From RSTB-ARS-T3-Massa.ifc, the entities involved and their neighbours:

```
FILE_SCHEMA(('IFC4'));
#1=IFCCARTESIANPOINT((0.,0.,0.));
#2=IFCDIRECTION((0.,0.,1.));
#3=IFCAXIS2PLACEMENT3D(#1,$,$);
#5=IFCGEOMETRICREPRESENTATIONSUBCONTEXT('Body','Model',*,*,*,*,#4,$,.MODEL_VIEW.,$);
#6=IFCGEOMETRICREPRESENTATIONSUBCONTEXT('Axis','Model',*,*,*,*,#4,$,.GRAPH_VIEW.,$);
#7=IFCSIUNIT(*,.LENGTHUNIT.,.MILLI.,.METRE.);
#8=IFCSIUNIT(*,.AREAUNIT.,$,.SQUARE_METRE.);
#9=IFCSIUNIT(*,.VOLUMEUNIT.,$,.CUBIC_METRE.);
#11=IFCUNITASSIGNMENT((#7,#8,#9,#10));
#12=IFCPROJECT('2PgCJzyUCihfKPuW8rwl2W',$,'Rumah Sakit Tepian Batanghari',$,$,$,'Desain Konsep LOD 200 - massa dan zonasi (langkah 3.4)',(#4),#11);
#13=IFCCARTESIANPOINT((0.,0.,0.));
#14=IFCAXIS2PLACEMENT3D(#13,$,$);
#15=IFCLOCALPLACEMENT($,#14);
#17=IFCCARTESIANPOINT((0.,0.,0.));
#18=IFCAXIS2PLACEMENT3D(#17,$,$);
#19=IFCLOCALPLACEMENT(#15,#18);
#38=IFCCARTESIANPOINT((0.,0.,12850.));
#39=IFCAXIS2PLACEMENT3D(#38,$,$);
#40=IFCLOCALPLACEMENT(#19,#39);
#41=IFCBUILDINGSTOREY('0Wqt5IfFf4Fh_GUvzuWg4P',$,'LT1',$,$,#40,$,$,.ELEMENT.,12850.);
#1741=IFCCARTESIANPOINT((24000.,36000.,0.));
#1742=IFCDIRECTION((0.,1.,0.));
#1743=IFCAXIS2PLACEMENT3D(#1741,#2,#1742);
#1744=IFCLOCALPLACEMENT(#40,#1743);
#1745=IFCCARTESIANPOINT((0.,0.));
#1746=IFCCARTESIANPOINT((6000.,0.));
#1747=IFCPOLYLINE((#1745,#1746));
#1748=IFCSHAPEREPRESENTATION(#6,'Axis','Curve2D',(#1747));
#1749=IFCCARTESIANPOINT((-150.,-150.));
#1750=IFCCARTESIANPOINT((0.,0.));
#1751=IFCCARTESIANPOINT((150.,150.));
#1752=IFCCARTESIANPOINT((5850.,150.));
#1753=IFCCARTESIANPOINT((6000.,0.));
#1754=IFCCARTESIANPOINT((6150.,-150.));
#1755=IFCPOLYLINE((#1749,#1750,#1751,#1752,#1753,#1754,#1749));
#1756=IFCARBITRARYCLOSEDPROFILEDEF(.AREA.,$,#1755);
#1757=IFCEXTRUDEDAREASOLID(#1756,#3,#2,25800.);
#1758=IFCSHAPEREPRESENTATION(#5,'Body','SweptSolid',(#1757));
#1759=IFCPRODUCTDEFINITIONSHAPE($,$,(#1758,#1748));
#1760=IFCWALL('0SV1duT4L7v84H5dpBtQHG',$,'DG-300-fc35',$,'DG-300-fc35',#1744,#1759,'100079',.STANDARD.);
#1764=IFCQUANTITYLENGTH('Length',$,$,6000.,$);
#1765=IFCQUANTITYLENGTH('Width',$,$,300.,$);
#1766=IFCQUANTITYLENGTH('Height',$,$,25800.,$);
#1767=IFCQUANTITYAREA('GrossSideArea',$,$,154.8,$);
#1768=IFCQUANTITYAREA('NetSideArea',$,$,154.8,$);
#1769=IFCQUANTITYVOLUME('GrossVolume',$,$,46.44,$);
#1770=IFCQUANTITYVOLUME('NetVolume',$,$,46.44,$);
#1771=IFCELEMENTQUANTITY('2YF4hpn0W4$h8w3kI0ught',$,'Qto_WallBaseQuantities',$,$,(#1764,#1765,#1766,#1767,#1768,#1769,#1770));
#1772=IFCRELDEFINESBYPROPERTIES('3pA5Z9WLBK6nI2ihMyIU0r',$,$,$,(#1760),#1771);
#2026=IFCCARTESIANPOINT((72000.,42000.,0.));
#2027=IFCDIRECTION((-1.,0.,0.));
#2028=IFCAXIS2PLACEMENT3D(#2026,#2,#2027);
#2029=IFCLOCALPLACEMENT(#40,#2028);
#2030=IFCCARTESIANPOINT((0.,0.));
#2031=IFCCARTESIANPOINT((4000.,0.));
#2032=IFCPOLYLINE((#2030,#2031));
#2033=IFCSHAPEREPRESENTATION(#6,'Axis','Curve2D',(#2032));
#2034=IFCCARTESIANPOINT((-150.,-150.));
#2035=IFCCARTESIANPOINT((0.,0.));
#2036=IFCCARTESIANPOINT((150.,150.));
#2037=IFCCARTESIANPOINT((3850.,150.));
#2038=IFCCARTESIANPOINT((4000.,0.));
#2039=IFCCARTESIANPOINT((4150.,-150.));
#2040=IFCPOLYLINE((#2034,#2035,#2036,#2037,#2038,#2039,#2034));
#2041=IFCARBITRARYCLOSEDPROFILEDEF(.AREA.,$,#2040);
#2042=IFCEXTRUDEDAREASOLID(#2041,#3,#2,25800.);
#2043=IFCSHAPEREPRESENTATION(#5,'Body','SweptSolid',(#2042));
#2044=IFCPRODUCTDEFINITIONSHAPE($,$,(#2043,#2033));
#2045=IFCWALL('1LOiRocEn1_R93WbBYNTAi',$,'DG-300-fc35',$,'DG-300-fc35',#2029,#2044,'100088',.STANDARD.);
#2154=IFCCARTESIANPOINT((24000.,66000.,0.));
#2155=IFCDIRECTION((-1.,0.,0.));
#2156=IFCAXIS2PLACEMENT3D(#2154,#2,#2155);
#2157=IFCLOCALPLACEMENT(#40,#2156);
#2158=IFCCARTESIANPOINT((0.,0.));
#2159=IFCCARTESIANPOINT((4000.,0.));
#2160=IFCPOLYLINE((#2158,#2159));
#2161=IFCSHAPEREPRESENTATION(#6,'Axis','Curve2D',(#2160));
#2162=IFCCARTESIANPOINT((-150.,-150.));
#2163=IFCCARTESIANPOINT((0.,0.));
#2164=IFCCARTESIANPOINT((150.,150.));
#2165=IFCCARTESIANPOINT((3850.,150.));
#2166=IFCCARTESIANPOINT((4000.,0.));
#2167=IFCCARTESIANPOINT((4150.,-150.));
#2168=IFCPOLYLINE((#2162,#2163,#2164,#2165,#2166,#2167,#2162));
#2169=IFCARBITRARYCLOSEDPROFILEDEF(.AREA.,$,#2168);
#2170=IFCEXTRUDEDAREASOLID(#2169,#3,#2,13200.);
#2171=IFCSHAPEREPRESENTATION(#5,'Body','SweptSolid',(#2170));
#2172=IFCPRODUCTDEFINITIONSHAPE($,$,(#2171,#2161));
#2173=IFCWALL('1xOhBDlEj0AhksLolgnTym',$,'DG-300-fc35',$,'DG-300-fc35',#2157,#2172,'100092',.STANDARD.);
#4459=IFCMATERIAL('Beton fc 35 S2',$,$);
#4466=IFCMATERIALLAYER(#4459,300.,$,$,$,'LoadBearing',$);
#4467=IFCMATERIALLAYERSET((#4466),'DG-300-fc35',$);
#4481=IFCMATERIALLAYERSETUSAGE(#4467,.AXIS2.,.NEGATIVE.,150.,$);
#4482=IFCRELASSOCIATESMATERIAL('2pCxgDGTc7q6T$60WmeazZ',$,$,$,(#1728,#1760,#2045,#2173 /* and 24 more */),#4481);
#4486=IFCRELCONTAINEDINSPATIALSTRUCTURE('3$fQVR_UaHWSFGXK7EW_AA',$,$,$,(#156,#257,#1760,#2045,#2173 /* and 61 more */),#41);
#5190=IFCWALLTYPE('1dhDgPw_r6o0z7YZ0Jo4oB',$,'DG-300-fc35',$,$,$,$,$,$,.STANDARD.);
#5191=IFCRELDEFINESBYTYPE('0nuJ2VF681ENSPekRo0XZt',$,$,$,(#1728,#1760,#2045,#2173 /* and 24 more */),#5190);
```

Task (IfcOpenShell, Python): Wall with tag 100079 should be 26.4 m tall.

```python
import ifcopenshell
import ifcopenshell.api.pset
import ifcopenshell.geom
import ifcopenshell.util.element
import ifcopenshell.util.representation
import ifcopenshell.util.shape
import ifcopenshell.util.unit

model = ifcopenshell.open("RSTB-ARS-T3-Massa.ifc")
unit_scale = ifcopenshell.util.unit.calculate_unit_scale(model)
area_scale = ifcopenshell.util.unit.calculate_unit_scale(model, "AREAUNIT")
volume_scale = ifcopenshell.util.unit.calculate_unit_scale(model, "VOLUMEUNIT")
settings = ifcopenshell.geom.settings()


def volume(element):
    """Net volume in cubic metres, openings subtracted."""
    shape = ifcopenshell.geom.create_shape(settings, element)
    return ifcopenshell.util.shape.get_volume(shape.geometry)


wall = model.by_id(1760)
before = volume(wall)

body = ifcopenshell.util.representation.get_representation(wall, "Model", "Body")
solid = body.Items[0]
old_height = solid.Depth
solid.Depth = 26400.0
after = volume(wall)
thickness = 0.3  # wall thickness in metres

# Update the stored height, areas and volumes.
qto = model.by_id(ifcopenshell.util.element.get_pset(wall, "Qto_WallBaseQuantities", should_inherit=False)["id"])
ifcopenshell.api.pset.edit_qto(model, qto=qto, properties={
    "Height": solid.Depth,
    "GrossSideArea": ifcopenshell.util.element.get_pset(wall, "Qto_WallBaseQuantities", "GrossSideArea") * solid.Depth / old_height,
    "NetSideArea": after / thickness / area_scale,
    "GrossVolume": ifcopenshell.util.element.get_pset(wall, "Qto_WallBaseQuantities", "GrossVolume") * solid.Depth / old_height,
    "NetVolume": after / volume_scale,
})

print(f"height {old_height:g} -> {solid.Depth:g}, volume {before:.3f} -> {after:.3f} m3")

model.write("RSTB-ARS-T3-Massa_updated.ifc")
```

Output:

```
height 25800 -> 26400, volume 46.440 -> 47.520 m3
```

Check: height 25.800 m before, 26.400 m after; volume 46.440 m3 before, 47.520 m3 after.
